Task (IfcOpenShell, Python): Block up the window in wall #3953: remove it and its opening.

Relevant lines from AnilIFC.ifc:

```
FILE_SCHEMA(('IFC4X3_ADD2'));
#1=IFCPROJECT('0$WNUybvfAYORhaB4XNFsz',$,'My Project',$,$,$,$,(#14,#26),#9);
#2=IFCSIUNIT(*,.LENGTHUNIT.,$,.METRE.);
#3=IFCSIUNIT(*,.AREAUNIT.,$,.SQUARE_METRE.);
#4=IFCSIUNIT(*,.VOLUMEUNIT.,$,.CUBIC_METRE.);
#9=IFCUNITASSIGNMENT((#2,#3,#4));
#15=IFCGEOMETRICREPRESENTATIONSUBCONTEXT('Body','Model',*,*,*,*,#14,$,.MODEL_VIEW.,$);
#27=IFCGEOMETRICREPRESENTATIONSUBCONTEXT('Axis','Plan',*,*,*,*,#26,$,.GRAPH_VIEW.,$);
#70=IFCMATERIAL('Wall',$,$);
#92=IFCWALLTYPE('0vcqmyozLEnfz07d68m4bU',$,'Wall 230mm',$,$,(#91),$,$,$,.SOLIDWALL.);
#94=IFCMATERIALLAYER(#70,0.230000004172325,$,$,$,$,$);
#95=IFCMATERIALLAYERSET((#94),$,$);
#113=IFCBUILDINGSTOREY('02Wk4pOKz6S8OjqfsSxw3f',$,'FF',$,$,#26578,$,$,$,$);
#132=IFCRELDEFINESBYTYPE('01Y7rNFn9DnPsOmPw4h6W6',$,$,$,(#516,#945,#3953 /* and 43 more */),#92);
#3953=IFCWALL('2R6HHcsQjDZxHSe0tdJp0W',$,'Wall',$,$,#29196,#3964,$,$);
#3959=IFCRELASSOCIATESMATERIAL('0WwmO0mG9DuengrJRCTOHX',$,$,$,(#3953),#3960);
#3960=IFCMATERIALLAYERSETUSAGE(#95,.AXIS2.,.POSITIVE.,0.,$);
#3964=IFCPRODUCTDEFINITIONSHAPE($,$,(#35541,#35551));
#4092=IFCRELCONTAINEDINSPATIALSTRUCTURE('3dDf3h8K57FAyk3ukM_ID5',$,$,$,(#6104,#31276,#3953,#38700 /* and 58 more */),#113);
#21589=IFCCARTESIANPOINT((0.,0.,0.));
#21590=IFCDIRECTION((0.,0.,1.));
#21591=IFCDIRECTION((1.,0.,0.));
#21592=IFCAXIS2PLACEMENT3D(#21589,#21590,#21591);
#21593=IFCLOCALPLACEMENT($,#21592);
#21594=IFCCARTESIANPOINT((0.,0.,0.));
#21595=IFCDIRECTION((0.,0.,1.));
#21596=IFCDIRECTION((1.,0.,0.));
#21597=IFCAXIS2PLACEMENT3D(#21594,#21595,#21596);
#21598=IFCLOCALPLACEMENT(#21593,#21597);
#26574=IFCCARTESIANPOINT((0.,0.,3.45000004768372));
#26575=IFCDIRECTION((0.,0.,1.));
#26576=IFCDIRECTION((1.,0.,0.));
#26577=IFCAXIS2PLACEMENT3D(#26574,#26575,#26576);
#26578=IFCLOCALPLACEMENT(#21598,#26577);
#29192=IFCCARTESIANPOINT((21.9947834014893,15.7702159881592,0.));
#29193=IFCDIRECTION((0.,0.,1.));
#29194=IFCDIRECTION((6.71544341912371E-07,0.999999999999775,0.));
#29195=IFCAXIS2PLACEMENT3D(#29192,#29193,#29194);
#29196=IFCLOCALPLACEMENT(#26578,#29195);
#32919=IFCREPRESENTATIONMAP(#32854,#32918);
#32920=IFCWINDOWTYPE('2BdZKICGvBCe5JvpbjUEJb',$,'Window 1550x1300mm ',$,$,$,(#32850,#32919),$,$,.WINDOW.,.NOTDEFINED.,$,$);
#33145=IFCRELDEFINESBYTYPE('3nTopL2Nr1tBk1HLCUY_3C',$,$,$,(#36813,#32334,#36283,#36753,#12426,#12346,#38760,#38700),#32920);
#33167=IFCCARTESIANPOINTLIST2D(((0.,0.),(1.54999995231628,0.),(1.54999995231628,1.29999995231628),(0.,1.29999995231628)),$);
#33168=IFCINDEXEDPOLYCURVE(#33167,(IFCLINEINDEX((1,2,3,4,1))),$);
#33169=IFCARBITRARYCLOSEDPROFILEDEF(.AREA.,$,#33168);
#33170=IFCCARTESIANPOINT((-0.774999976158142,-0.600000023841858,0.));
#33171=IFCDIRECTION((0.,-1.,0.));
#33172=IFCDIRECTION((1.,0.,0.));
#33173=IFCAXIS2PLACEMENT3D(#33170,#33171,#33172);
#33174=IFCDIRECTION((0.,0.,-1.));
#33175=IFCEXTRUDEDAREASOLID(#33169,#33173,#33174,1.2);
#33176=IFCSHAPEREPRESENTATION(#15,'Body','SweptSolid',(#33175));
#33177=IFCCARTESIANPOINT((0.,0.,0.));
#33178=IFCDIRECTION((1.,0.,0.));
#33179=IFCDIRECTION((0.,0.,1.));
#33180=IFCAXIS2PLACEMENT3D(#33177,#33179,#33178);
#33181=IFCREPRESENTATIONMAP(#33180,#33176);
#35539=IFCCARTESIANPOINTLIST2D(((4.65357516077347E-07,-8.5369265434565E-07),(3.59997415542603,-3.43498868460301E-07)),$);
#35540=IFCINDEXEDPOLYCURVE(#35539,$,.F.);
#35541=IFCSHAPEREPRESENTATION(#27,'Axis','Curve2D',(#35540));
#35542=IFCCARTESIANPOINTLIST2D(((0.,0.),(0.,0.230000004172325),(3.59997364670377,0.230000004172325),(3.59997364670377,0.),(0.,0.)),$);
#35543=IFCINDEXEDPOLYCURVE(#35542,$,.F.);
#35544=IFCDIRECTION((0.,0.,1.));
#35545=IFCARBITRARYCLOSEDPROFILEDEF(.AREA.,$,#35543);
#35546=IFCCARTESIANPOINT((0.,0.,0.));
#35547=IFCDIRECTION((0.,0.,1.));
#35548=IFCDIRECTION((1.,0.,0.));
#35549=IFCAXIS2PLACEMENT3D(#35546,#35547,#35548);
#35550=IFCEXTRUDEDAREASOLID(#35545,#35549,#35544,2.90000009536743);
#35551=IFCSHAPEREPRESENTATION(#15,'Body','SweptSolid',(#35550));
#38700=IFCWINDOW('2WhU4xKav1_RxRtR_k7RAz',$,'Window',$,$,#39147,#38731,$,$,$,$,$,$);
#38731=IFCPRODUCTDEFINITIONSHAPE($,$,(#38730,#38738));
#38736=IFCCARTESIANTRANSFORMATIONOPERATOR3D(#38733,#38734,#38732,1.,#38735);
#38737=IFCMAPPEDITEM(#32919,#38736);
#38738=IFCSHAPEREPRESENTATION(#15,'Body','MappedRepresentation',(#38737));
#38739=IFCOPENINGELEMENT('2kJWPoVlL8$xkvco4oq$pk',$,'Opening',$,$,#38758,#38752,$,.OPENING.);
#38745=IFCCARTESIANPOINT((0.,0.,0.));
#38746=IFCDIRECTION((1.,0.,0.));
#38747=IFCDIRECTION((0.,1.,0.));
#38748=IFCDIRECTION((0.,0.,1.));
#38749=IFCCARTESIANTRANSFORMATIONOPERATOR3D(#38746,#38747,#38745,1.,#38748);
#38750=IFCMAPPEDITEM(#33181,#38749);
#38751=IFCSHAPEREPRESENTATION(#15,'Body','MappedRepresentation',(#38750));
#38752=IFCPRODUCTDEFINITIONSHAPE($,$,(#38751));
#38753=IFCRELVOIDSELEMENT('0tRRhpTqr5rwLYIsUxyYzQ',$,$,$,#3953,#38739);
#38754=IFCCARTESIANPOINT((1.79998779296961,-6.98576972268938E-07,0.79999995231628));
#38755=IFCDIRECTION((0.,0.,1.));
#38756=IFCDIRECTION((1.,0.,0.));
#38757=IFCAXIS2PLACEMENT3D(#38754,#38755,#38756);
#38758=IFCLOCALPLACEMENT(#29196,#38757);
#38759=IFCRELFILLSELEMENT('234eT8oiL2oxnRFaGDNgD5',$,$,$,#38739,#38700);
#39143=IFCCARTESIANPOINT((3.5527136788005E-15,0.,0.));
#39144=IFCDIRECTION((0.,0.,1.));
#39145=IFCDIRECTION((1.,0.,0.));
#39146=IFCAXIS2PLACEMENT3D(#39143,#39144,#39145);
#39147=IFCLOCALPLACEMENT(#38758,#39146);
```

```python
import ifcopenshell
import ifcopenshell.api.feature
import ifcopenshell.api.root
import ifcopenshell.geom
import ifcopenshell.util.shape

model = ifcopenshell.open("AnilIFC.ifc")
settings = ifcopenshell.geom.settings()


def volume(element):
    """Net volume in cubic metres, openings subtracted."""
    shape = ifcopenshell.geom.create_shape(settings, element)
    return ifcopenshell.util.shape.get_volume(shape.geometry)


window = model.by_guid("2WhU4xKav1_RxRtR_k7RAz")
opening = window.FillsVoids[0].RelatingOpeningElement
wall = opening.VoidsElements[0].RelatingBuildingElement
before = volume(wall)

ifcopenshell.api.root.remove_product(model, product=window)
ifcopenshell.api.feature.remove_feature(model, feature=opening)

after = volume(wall)

print(f"wall volume {before:.3f} -> {after:.3f} m3")

model.write("AnilIFC_edited.ifc")
```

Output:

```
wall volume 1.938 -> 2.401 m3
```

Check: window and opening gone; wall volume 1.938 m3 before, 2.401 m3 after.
